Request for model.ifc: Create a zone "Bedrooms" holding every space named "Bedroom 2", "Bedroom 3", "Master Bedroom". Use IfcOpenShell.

First a look at what the model holds.

```python
import ifcopenshell

model = ifcopenshell.open("model.ifc")
print(model.schema)
seen = {}
for space in model.by_type("IfcSpace"):
    seen[space.LongName] = seen.get(space.LongName, 0) + 1
for name, count in sorted(seen.items(), key=str):
    print(count, "x", name)
print("zones:", [z.Name for z in model.by_type("IfcZone")][:20])
```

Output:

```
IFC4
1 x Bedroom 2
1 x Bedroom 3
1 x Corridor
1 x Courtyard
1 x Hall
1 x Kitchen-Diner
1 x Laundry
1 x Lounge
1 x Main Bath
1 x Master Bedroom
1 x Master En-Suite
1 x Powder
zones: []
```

```python
import ifcopenshell
import ifcopenshell.api.group
import ifcopenshell.api.root

model = ifcopenshell.open("model.ifc")

names = {"Bedroom 2", "Bedroom 3", "Master Bedroom"}
spaces = [s for s in model.by_type("IfcSpace") if s.LongName in names]

zone = ifcopenshell.api.root.create_entity(model, ifc_class="IfcZone", name="Bedrooms")
ifcopenshell.api.group.assign_group(model, products=spaces, group=zone)
print(len(spaces), "spaces in", zone.Name)

model.write("model_rev.ifc")
```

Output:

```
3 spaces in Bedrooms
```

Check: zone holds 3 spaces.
